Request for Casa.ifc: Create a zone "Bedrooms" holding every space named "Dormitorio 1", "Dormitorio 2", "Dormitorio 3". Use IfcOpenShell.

First a look at what the model holds.

```python
import ifcopenshell

model = ifcopenshell.open("Casa.ifc")
print(model.schema)
seen = {}
for space in model.by_type("IfcSpace"):
    seen[space.LongName] = seen.get(space.LongName, 0) + 1
for name, count in sorted(seen.items(), key=str):
    print(count, "x", name)
print("zones:", [z.Name for z in model.by_type("IfcZone")][:20])
```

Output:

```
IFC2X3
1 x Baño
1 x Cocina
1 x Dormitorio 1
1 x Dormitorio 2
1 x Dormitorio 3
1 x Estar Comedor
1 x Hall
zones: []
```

```python
import ifcopenshell
import ifcopenshell.api.group
import ifcopenshell.api.root

model = ifcopenshell.open("Casa.ifc")

names = {"Dormitorio 1", "Dormitorio 2", "Dormitorio 3"}
spaces = [s for s in model.by_type("IfcSpace") if s.LongName in names]

zone = ifcopenshell.api.root.create_entity(model, ifc_class="IfcZone", name="Bedrooms")
ifcopenshell.api.group.assign_group(model, products=spaces, group=zone)
print(len(spaces), "spaces in", zone.Name)

model.write("Casa_edited.ifc")
```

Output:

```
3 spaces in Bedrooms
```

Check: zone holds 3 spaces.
